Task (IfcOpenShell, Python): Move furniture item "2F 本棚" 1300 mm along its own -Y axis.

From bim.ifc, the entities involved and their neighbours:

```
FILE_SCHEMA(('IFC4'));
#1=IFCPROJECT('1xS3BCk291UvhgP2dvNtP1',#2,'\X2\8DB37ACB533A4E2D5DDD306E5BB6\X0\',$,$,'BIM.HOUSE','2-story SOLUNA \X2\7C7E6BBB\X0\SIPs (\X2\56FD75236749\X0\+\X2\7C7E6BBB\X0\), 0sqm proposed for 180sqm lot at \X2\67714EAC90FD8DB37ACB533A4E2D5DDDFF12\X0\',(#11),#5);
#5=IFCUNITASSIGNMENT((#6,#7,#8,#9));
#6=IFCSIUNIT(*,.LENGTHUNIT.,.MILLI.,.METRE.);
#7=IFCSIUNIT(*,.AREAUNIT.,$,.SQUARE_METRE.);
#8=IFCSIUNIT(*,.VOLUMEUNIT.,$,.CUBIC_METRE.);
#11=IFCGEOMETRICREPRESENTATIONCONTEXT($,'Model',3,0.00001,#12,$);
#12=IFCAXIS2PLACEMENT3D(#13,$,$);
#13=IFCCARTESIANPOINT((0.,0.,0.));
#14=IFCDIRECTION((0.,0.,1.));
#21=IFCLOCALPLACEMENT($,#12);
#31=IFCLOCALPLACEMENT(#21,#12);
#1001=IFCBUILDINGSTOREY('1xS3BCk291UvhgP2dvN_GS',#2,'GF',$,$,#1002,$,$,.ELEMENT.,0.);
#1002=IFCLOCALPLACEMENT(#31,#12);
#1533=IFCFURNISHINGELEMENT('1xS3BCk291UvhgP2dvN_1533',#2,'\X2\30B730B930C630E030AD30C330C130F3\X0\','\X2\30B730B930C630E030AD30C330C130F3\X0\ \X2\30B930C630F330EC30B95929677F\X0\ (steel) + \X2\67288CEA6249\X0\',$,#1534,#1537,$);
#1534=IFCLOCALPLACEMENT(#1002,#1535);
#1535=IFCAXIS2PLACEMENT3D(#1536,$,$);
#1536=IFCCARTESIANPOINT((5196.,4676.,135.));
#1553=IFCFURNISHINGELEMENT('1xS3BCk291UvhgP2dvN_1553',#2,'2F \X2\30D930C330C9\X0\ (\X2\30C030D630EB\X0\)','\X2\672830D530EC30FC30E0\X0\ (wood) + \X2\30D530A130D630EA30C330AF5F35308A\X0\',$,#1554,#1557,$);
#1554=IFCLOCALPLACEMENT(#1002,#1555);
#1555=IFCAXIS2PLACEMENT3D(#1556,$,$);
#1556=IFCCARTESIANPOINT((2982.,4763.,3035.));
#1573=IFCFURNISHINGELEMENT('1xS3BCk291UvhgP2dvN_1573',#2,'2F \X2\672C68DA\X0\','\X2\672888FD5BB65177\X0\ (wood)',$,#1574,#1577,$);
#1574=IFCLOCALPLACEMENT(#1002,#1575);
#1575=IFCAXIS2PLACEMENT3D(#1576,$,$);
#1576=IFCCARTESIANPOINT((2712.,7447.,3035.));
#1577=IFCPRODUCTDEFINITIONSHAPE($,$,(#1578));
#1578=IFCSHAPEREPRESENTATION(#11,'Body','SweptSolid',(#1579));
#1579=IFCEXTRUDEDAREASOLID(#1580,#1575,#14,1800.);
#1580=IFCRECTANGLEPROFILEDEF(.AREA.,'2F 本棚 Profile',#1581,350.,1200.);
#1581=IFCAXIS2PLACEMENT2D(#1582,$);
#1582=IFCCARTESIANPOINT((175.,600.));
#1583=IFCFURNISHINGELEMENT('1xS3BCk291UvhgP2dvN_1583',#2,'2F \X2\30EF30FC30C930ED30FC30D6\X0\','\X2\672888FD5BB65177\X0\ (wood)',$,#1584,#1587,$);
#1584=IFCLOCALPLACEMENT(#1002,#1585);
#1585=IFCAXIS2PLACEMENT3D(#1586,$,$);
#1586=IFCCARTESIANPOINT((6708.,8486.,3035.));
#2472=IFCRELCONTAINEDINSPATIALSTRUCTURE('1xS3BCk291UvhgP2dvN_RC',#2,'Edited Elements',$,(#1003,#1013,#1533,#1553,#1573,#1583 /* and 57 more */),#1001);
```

```python
import ifcopenshell
import ifcopenshell.api.geometry
import ifcopenshell.util.placement

model = ifcopenshell.open("bim.ifc")

item = model.by_guid("1xS3BCk291UvhgP2dvN_1573")
matrix = ifcopenshell.util.placement.get_local_placement(item.ObjectPlacement)
matrix[:3, 3] -= matrix[:3, 1] * 1300.0
ifcopenshell.api.geometry.edit_object_placement(model, product=item, matrix=matrix, is_si=False)

print(ifcopenshell.util.placement.get_local_placement(item.ObjectPlacement).round(3) + 0.0)

model.write("bim_edited.ifc")
```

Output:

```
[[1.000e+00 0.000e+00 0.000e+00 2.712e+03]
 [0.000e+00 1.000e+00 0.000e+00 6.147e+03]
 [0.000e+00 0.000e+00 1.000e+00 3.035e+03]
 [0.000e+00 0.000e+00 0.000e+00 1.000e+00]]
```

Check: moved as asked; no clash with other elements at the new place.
